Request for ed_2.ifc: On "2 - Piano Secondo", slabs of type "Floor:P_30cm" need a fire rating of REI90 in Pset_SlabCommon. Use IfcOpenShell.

First a look at what the model holds.

```python
import ifcopenshell
import ifcopenshell.util.element

model = ifcopenshell.open("ed_2.ifc")
print(model.schema)
storey = next(s for s in model.by_type("IfcBuildingStorey") if s.Name == "2 - Piano Secondo")
slabs = [e for e in ifcopenshell.util.element.get_decomposition(storey) if e.is_a("IfcSlab")]
seen = {}
for e in slabs:
    element_type = ifcopenshell.util.element.get_type(e)
    key = (element_type.Name if element_type != e and element_type else None, ifcopenshell.util.element.get_pset(e, "Pset_SlabCommon", "FireRating"))
    seen[key] = seen.get(key, 0) + 1
for (name, value), count in sorted(seen.items(), key=str):
    print(count, "x", name, "|", value)
```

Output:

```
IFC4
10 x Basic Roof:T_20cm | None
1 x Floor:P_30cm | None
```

```python
import ifcopenshell
import ifcopenshell.api.pset
import ifcopenshell.util.element

model = ifcopenshell.open("ed_2.ifc")

storey = next(s for s in model.by_type("IfcBuildingStorey") if s.Name == "2 - Piano Secondo")
slabs = [e for e in ifcopenshell.util.element.get_decomposition(storey) if e.is_a("IfcSlab")]

count = 0
for e in slabs:
    element_type = ifcopenshell.util.element.get_type(e)
    if element_type in (None, e) or element_type.Name != "Floor:P_30cm":
        continue
    # add_pset returns the element's existing set when there is one.
    pset = ifcopenshell.api.pset.add_pset(model, product=e, name="Pset_SlabCommon")
    ifcopenshell.api.pset.edit_pset(model, pset=pset, properties={"FireRating": "REI90"})
    count += 1

print(count, "slabs updated")

model.write("ed_2-out.ifc")
```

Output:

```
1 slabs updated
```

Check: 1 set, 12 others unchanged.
